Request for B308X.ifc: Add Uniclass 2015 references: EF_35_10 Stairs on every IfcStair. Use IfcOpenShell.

First a look at what the model holds.

```python
import ifcopenshell

model = ifcopenshell.open("B308X.ifc")
print(model.schema)
print("classifications:", [c.Name for c in model.by_type("IfcClassification")])
for ifc_class in ("IfcDoor", "IfcRoof", "IfcStair", "IfcWall", "IfcWindow"):
    print(ifc_class, len(model.by_type(ifc_class)))
```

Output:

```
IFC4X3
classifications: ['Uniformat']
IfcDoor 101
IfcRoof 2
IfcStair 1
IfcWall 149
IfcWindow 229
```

```python
import ifcopenshell
import ifcopenshell.api.classification

model = ifcopenshell.open("B308X.ifc")

system = ifcopenshell.api.classification.add_classification(model, classification="Uniclass 2015")

codes = {
    "IfcStair": ("EF_35_10", "Stairs"),
}
for ifc_class, (code, name) in codes.items():
    products = model.by_type(ifc_class)
    ifcopenshell.api.classification.add_reference(
        model, products=products, classification=system, identification=code, name=name
    )
    print(code, len(products))

model.write("B308X_rev.ifc")
```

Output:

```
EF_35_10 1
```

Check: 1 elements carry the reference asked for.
